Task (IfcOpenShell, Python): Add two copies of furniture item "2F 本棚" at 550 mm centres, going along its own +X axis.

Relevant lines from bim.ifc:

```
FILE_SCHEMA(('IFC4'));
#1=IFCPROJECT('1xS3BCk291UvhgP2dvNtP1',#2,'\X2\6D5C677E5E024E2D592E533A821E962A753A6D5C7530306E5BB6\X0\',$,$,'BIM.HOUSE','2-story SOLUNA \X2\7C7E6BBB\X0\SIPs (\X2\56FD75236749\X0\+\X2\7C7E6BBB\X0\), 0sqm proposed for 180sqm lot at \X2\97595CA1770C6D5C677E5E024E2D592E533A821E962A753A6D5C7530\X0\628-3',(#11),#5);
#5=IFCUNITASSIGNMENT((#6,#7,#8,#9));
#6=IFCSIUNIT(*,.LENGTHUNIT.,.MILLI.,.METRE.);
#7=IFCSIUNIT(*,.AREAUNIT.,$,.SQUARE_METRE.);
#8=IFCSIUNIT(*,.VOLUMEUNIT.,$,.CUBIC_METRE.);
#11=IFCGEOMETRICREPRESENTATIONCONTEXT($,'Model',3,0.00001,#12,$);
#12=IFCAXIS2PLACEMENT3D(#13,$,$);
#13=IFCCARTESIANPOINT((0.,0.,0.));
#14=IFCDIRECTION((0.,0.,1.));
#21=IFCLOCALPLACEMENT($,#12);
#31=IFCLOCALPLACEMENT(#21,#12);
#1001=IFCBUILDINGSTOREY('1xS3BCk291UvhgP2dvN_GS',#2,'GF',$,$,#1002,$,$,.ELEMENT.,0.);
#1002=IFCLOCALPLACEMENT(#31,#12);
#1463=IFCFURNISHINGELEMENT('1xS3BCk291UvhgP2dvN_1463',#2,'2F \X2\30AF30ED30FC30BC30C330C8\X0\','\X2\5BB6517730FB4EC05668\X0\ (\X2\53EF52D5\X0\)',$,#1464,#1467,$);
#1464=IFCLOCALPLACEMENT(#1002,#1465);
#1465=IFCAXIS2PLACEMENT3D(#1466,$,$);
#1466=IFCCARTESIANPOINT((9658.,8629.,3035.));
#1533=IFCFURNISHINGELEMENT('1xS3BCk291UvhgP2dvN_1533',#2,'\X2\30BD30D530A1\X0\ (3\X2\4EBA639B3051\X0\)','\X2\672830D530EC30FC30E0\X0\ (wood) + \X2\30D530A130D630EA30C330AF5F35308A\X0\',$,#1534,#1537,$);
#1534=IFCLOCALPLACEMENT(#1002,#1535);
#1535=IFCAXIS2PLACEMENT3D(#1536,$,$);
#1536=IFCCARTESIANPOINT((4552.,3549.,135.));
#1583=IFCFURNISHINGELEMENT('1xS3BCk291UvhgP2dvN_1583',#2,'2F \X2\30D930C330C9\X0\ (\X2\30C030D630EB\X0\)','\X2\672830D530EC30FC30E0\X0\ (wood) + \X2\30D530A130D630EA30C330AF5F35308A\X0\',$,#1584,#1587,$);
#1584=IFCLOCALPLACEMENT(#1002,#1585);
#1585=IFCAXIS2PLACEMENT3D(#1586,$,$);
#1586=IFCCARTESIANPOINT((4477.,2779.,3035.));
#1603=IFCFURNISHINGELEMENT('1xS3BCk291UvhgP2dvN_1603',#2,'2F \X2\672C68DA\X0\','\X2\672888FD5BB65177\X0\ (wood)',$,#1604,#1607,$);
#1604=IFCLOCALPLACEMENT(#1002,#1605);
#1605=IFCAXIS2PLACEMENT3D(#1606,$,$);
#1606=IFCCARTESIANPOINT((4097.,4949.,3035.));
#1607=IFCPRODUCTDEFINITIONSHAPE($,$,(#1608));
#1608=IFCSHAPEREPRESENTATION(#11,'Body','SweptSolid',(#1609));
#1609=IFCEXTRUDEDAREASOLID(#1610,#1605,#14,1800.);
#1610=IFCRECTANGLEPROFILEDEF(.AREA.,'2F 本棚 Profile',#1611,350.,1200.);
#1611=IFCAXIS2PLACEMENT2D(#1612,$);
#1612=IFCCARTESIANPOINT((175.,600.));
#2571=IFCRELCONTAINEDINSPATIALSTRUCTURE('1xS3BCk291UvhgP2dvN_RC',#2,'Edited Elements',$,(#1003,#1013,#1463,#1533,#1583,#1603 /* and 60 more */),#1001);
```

```python
import ifcopenshell
import ifcopenshell.api.geometry
import ifcopenshell.api.root
import ifcopenshell.util.element
import ifcopenshell.util.placement

model = ifcopenshell.open("bim.ifc")


def reuse_history(source, copy):
    """copy_class also copies each property set's owner history, people and application; keep the originals."""
    for rel in copy.IsDefinedBy:
        if rel.is_a("IfcRelDefinesByProperties") and (history := rel.RelatingPropertyDefinition.OwnerHistory):
            rel.RelatingPropertyDefinition.OwnerHistory = source.OwnerHistory
            ifcopenshell.util.element.remove_deep2(model, history)


source = model.by_guid("1xS3BCk291UvhgP2dvN_1603")
base = ifcopenshell.util.placement.get_local_placement(source.ObjectPlacement)
step = base[:3, 0] * 550.0

for i in range(1, 3):
    copy = ifcopenshell.api.root.copy_class(model, product=source)
    copy.Representation = ifcopenshell.util.element.copy_deep(
        model, source.Representation, exclude=["IfcGeometricRepresentationContext", "IfcRepresentationMap"]
    )
    reuse_history(source, copy)
    matrix = base.copy()
    matrix[:3, 3] += i * step
    print("added at", matrix[:3, 3].round(3) + 0.0)
    ifcopenshell.api.geometry.edit_object_placement(model, product=copy, matrix=matrix, is_si=False)

model.write("bim_v2.ifc")
```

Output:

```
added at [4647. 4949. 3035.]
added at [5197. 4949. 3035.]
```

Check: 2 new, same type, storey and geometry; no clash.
